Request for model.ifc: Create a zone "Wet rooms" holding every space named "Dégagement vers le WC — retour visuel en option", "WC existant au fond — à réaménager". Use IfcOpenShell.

First a look at what the model holds.

```python
import ifcopenshell

model = ifcopenshell.open("model.ifc")
print(model.schema)
seen = {}
for space in model.by_type("IfcSpace"):
    seen[space.LongName] = seen.get(space.LongName, 0) + 1
for name, count in sorted(seen.items(), key=str):
    print(count, "x", name)
print("zones:", [z.Name for z in model.by_type("IfcZone")][:20])
```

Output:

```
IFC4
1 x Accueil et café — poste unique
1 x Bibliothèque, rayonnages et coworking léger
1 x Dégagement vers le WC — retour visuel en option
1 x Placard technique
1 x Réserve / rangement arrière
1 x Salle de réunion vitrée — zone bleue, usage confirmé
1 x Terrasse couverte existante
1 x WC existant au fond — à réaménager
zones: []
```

```python
import ifcopenshell
import ifcopenshell.api.group
import ifcopenshell.api.root

model = ifcopenshell.open("model.ifc")

names = {"Dégagement vers le WC — retour visuel en option", "WC existant au fond — à réaménager"}
spaces = [s for s in model.by_type("IfcSpace") if s.LongName in names]

zone = ifcopenshell.api.root.create_entity(model, ifc_class="IfcZone", name="Wet rooms")
ifcopenshell.api.group.assign_group(model, products=spaces, group=zone)
print(len(spaces), "spaces in", zone.Name)

model.write("model_edited.ifc")
```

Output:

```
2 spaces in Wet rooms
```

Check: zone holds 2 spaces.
